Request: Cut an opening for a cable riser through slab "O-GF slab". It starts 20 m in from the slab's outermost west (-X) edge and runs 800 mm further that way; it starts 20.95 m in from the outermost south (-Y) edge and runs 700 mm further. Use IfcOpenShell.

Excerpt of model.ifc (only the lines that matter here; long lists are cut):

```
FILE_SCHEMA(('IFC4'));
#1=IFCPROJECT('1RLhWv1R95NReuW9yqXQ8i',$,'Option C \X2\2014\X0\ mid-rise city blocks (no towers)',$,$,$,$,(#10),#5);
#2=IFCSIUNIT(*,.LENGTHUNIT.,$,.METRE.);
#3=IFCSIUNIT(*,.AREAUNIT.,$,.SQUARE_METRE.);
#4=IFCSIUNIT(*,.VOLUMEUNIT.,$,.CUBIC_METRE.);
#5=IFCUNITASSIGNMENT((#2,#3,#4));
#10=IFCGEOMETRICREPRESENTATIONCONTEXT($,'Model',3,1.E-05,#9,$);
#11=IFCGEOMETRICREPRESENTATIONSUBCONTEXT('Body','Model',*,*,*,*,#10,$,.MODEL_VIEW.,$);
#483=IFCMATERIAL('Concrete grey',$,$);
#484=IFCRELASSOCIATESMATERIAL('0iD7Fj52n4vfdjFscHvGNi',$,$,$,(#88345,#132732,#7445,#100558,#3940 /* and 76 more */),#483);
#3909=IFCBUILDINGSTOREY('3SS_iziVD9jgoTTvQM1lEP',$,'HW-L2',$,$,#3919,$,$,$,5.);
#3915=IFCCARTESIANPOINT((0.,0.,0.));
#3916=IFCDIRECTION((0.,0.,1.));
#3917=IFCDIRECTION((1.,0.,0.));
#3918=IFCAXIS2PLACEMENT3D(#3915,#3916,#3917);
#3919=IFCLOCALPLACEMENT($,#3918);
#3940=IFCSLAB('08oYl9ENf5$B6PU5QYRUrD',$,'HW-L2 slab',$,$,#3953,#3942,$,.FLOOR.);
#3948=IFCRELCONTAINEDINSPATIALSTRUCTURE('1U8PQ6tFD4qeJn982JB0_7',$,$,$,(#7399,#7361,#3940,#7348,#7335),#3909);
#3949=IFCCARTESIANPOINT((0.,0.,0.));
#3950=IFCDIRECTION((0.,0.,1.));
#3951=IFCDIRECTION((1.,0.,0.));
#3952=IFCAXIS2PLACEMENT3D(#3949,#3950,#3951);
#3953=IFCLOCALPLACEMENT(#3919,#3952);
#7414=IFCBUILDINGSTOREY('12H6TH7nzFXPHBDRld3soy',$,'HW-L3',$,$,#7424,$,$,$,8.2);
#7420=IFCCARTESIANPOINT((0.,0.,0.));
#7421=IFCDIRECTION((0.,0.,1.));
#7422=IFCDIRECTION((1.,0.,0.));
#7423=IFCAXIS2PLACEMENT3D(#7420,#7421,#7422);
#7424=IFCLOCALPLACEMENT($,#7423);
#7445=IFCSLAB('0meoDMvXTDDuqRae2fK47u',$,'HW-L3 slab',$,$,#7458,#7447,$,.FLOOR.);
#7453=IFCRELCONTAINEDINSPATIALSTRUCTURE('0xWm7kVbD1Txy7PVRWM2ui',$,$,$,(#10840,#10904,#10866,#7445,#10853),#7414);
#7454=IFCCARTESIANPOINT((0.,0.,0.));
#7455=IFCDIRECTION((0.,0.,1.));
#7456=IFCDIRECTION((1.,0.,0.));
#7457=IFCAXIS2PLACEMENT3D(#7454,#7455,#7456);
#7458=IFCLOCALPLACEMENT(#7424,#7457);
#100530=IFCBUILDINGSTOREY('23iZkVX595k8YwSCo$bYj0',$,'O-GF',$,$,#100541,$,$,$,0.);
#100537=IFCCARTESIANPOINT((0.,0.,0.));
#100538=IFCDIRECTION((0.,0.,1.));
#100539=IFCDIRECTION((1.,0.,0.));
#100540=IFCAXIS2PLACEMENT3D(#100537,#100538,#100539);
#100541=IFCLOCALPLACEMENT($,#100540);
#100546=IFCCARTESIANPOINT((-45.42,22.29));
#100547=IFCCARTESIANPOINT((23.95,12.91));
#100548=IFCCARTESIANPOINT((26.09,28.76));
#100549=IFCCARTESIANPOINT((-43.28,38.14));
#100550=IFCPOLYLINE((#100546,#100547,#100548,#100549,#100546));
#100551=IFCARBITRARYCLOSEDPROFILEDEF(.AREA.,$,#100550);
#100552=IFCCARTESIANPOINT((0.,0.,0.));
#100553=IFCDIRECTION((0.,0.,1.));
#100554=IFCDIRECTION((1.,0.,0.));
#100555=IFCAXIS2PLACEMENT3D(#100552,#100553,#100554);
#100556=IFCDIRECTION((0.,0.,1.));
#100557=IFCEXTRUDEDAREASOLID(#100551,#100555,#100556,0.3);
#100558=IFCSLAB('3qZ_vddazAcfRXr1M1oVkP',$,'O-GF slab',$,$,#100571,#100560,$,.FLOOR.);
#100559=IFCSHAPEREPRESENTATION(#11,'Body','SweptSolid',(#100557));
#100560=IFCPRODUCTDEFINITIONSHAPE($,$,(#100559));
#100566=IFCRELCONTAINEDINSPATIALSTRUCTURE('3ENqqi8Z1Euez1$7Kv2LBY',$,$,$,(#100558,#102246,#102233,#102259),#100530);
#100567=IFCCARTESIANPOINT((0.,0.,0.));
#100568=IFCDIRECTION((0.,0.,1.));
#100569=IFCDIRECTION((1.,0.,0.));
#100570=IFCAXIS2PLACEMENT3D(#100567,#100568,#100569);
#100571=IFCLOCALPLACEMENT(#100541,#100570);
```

```python
import numpy as np
import ifcopenshell
import ifcopenshell.api.feature
import ifcopenshell.api.geometry
import ifcopenshell.api.root
import ifcopenshell.geom
import ifcopenshell.util.placement
import ifcopenshell.util.representation
import ifcopenshell.util.shape
import ifcopenshell.util.unit

model = ifcopenshell.open("model.ifc")
unit_scale = ifcopenshell.util.unit.calculate_unit_scale(model)
settings = ifcopenshell.geom.settings()


def volume(element):
    """Net volume in cubic metres, openings subtracted."""
    shape = ifcopenshell.geom.create_shape(settings, element)
    return ifcopenshell.util.shape.get_volume(shape.geometry)


slab = model.by_guid("3qZ_vddazAcfRXr1M1oVkP")
before = volume(slab)

# Extent in the slab's own axes, in metres. The edges named are its -X and -Y sides.
slab_shape = ifcopenshell.geom.create_shape(settings, slab)
vertices = ifcopenshell.util.shape.get_vertices(slab_shape.geometry)
x_min, y_min, bottom = vertices.min(axis=0)
top = vertices[:, 2].max()

opening = ifcopenshell.api.root.create_entity(model, ifc_class="IfcOpeningElement", name="Cable riser opening", predefined_type="OPENING")
context = ifcopenshell.util.representation.get_context(model, "Model", "Body", "MODEL_VIEW")
width, depth = 0.8, 0.7
outline = [(0.0, 0.0), (width, 0.0), (width, depth), (0.0, depth), (0.0, 0.0)]
# Overshoot both faces by 50 mm so the cut is clean.
shape = ifcopenshell.api.geometry.add_slab_representation(
    model, context=context, depth=top - bottom + 0.1, polyline=outline
)
ifcopenshell.api.geometry.assign_representation(model, product=opening, representation=shape)

matrix = ifcopenshell.util.placement.get_local_placement(slab.ObjectPlacement)
matrix[:, 3] = matrix @ np.append(np.array([x_min + 20, y_min + 20.95, bottom - 0.05]) / unit_scale, 1.0)
ifcopenshell.api.geometry.edit_object_placement(model, product=opening, matrix=matrix, is_si=False)
ifcopenshell.api.feature.add_feature(model, feature=opening, element=slab)

after = volume(slab)

print(f"slab volume {before:.3f} -> {after:.3f} m3")

model.write("model_v2.ifc")
```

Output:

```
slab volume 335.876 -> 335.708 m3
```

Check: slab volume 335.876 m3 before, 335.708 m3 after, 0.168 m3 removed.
